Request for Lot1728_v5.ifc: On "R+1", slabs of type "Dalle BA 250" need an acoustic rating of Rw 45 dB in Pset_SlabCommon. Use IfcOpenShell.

First a look at what the model holds.

```python
import ifcopenshell
import ifcopenshell.util.element

model = ifcopenshell.open("Lot1728_v5.ifc")
print(model.schema)
storey = next(s for s in model.by_type("IfcBuildingStorey") if s.Name == "R+1")
slabs = [e for e in ifcopenshell.util.element.get_decomposition(storey) if e.is_a("IfcSlab")]
seen = {}
for e in slabs:
    element_type = ifcopenshell.util.element.get_type(e)
    key = (element_type.Name if element_type != e and element_type else None, ifcopenshell.util.element.get_pset(e, "Pset_SlabCommon", "AcousticRating"))
    seen[key] = seen.get(key, 0) + 1
for (name, value), count in sorted(seen.items(), key=str):
    print(count, "x", name, "|", value)
```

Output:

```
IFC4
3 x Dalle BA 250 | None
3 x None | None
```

```python
import ifcopenshell
import ifcopenshell.api.pset
import ifcopenshell.util.element

model = ifcopenshell.open("Lot1728_v5.ifc")

storey = next(s for s in model.by_type("IfcBuildingStorey") if s.Name == "R+1")
slabs = [e for e in ifcopenshell.util.element.get_decomposition(storey) if e.is_a("IfcSlab")]

count = 0
for e in slabs:
    element_type = ifcopenshell.util.element.get_type(e)
    if element_type in (None, e) or element_type.Name != "Dalle BA 250":
        continue
    # add_pset returns the element's existing set when there is one.
    pset = ifcopenshell.api.pset.add_pset(model, product=e, name="Pset_SlabCommon")
    ifcopenshell.api.pset.edit_pset(model, pset=pset, properties={"AcousticRating": "Rw 45 dB"})
    count += 1

print(count, "slabs updated")

model.write("Lot1728_v5_v2.ifc")
```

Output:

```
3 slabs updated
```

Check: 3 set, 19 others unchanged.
